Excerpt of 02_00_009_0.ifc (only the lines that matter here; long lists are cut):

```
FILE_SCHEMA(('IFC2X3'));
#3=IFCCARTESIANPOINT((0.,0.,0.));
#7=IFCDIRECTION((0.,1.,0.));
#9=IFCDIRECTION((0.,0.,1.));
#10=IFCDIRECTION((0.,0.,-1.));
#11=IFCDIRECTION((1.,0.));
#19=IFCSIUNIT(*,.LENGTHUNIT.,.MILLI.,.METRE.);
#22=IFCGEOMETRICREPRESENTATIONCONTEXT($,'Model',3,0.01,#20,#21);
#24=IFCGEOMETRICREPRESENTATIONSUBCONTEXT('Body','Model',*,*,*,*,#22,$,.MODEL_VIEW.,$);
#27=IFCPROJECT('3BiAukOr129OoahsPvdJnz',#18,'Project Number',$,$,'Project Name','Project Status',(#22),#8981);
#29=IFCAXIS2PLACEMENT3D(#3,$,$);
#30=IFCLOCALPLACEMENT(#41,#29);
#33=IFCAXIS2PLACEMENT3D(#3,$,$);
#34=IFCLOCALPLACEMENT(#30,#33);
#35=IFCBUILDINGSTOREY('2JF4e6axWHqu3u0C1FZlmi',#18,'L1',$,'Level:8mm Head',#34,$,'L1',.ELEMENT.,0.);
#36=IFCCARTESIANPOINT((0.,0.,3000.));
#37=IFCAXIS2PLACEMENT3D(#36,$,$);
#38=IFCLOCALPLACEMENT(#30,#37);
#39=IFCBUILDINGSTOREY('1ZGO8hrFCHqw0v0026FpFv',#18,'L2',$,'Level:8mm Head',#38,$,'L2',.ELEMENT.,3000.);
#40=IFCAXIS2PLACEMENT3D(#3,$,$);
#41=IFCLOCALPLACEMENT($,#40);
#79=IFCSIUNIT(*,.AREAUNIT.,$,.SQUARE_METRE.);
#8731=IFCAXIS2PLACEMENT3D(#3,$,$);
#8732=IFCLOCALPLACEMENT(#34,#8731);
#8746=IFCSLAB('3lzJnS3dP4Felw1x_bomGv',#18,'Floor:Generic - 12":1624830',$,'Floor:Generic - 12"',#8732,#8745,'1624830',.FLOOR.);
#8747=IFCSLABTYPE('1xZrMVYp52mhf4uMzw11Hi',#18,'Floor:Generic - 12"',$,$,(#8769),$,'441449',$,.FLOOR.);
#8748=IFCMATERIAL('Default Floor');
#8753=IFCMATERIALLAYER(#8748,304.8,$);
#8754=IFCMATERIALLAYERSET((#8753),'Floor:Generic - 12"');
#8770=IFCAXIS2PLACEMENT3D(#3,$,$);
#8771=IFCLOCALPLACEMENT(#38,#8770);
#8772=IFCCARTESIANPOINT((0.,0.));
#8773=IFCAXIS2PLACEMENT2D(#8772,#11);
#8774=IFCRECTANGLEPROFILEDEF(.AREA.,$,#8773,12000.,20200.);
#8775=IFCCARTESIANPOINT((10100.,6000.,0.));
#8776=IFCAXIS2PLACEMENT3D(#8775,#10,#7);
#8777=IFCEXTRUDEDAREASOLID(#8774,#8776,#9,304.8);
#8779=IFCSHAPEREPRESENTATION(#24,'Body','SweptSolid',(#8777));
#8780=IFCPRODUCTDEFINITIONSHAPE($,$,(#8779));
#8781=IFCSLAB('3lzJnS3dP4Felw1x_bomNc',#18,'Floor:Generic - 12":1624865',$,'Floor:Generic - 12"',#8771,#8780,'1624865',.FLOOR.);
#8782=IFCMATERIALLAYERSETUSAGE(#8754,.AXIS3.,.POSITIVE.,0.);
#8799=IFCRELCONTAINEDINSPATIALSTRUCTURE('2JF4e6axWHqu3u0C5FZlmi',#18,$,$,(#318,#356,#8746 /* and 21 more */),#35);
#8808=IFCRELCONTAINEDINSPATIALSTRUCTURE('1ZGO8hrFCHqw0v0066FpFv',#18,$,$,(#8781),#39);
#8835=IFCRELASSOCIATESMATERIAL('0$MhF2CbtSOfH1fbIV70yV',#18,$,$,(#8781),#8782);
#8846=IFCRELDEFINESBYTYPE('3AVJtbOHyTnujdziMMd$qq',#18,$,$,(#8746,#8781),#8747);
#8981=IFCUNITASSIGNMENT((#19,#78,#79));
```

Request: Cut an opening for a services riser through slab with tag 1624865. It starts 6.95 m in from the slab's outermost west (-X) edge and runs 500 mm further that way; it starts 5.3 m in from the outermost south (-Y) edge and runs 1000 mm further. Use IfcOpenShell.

```python
import numpy as np
import ifcopenshell
import ifcopenshell.api.feature
import ifcopenshell.api.geometry
import ifcopenshell.api.root
import ifcopenshell.geom
import ifcopenshell.util.placement
import ifcopenshell.util.representation
import ifcopenshell.util.shape
import ifcopenshell.util.unit

model = ifcopenshell.open("02_00_009_0.ifc")
unit_scale = ifcopenshell.util.unit.calculate_unit_scale(model)
settings = ifcopenshell.geom.settings()


def volume(element):
    """Net volume in cubic metres, openings subtracted."""
    shape = ifcopenshell.geom.create_shape(settings, element)
    return ifcopenshell.util.shape.get_volume(shape.geometry)


slab = model.by_guid("3lzJnS3dP4Felw1x_bomNc")
before = volume(slab)

# Extent in the slab's own axes, in metres. The edges named are its -X and -Y sides.
slab_shape = ifcopenshell.geom.create_shape(settings, slab)
vertices = ifcopenshell.util.shape.get_vertices(slab_shape.geometry)
x_min, y_min, bottom = vertices.min(axis=0)
top = vertices[:, 2].max()

opening = ifcopenshell.api.root.create_entity(model, ifc_class="IfcOpeningElement", name="Services riser opening")
context = ifcopenshell.util.representation.get_context(model, "Model", "Body", "MODEL_VIEW")
width, depth = 0.5, 1
outline = [(0.0, 0.0), (width, 0.0), (width, depth), (0.0, depth), (0.0, 0.0)]
# Overshoot both faces by 50 mm so the cut is clean.
shape = ifcopenshell.api.geometry.add_slab_representation(
    model, context=context, depth=top - bottom + 0.1, polyline=outline
)
ifcopenshell.api.geometry.assign_representation(model, product=opening, representation=shape)

matrix = ifcopenshell.util.placement.get_local_placement(slab.ObjectPlacement)
matrix[:, 3] = matrix @ np.append(np.array([x_min + 6.95, y_min + 5.3, bottom - 0.05]) / unit_scale, 1.0)
ifcopenshell.api.geometry.edit_object_placement(model, product=opening, matrix=matrix, is_si=False)
ifcopenshell.api.feature.add_feature(model, feature=opening, element=slab)

after = volume(slab)

print(f"slab volume {before:.3f} -> {after:.3f} m3")

model.write("02_00_009_0_rev.ifc")
```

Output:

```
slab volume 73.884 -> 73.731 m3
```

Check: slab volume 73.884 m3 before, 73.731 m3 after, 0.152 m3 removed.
